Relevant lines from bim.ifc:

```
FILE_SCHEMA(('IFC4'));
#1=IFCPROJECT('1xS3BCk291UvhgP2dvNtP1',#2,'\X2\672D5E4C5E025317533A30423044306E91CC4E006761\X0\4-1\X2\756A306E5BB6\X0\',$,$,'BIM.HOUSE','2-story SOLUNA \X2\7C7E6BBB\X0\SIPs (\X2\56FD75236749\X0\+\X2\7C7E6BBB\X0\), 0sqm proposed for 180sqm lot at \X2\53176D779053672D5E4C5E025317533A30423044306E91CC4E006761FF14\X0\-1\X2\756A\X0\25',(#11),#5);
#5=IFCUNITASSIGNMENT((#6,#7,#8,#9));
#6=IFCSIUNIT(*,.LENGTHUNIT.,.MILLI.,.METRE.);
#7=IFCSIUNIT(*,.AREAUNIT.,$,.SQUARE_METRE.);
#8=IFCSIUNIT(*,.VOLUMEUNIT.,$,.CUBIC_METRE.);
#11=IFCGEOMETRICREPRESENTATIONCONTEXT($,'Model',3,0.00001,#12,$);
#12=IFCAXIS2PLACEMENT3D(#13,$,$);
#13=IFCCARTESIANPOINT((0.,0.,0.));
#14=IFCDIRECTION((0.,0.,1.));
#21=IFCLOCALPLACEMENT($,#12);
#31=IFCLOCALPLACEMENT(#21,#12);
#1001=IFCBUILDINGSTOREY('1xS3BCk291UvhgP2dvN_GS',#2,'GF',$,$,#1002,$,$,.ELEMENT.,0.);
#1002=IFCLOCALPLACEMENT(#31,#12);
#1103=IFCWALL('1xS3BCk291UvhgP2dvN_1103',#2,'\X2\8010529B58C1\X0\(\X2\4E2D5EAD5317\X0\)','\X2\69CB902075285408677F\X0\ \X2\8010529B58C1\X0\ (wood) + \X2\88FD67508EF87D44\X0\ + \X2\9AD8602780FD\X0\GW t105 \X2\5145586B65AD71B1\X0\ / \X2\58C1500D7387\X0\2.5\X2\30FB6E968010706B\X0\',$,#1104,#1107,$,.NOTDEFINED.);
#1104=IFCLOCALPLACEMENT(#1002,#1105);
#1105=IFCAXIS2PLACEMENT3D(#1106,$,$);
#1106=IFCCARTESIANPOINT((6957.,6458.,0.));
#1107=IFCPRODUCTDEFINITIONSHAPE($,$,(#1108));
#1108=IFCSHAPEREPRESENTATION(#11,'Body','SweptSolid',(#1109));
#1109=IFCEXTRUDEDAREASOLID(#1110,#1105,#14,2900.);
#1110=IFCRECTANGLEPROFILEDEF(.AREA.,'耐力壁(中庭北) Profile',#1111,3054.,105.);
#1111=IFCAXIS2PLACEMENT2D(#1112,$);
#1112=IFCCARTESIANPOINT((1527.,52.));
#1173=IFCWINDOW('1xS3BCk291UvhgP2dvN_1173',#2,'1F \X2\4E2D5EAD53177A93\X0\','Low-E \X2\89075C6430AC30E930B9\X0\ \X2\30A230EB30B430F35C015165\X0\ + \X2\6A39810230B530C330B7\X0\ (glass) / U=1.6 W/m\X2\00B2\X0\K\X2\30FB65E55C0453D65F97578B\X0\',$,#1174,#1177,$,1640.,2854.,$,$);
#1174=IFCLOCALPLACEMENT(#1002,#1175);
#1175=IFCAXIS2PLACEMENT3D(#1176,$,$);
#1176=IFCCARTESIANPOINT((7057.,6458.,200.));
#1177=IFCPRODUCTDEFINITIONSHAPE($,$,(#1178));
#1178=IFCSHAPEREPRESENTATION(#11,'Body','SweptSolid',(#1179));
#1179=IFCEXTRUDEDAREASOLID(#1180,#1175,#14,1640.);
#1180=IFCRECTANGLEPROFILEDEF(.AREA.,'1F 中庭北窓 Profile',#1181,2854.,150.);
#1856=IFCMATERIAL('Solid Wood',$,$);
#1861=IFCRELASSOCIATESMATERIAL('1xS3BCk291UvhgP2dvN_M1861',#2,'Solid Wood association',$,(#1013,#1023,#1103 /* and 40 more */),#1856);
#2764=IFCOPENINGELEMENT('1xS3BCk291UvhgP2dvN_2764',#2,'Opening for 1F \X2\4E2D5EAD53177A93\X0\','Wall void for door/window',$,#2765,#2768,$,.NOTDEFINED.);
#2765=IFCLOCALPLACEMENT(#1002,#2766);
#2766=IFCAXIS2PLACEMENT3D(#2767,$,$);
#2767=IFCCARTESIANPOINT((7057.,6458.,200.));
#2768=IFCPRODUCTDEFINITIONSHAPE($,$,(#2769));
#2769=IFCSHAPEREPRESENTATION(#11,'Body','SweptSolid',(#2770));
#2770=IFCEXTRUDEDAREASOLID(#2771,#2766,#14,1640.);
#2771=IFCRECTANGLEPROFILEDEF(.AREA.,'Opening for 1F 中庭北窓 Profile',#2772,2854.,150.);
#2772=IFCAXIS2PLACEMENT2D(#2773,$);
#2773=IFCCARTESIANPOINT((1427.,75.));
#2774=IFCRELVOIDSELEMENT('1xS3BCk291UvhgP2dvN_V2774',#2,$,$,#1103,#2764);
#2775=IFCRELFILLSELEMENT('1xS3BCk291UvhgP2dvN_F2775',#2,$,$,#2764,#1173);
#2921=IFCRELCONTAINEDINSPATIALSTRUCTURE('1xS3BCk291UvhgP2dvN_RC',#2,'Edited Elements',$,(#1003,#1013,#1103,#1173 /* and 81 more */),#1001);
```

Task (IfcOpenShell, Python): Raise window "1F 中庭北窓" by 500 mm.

```python
import numpy as np
import ifcopenshell
import ifcopenshell.api.geometry
import ifcopenshell.util.placement
import ifcopenshell.util.unit

model = ifcopenshell.open("bim.ifc")
unit_scale = ifcopenshell.util.unit.calculate_unit_scale(model)

window = model.by_guid("1xS3BCk291UvhgP2dvN_1173")
opening = window.FillsVoids[0].RelatingOpeningElement
dz = 500.0

shift = np.array([0.0, 0.0, dz])
# The window is not placed relative to its opening, so move both.
for product in (opening, window):
    matrix = ifcopenshell.util.placement.get_local_placement(product.ObjectPlacement)
    matrix[:3, 3] += shift
    ifcopenshell.api.geometry.edit_object_placement(model, product=product, matrix=matrix, is_si=False)

print(f"moved by {dz * unit_scale:+.3f} m")

model.write("bim_updated.ifc")
```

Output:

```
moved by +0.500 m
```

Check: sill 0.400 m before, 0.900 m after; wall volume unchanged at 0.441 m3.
